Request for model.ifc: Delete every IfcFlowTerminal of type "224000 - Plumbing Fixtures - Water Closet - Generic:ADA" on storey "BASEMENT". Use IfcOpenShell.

First a look at what the model holds.

```python
import ifcopenshell
import ifcopenshell.util.element

model = ifcopenshell.open("model.ifc")
print(model.schema)
storey = next(s for s in model.by_type("IfcBuildingStorey") if s.Name == "BASEMENT")
terminals = [e for e in ifcopenshell.util.element.get_decomposition(storey) if e.is_a("IfcFlowTerminal")]
seen = {}
for e in terminals:
    element_type = ifcopenshell.util.element.get_type(e)
    name = element_type.Name if element_type not in (None, e) else None
    seen[name] = seen.get(name, 0) + 1
for name, count in sorted(seen.items(), key=str):
    print(count, "x", name)
```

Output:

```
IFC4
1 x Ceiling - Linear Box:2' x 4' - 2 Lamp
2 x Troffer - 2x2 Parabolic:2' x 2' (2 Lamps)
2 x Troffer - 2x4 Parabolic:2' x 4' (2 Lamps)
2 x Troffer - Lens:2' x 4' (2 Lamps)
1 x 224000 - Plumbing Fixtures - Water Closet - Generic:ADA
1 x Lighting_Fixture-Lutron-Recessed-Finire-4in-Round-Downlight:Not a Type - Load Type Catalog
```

```python
import ifcopenshell
import ifcopenshell.api.root
import ifcopenshell.util.element

model = ifcopenshell.open("model.ifc")

storey = next(s for s in model.by_type("IfcBuildingStorey") if s.Name == "BASEMENT")
terminals = [e for e in ifcopenshell.util.element.get_decomposition(storey) if e.is_a("IfcFlowTerminal")]
targets = [e for e in terminals if (t := ifcopenshell.util.element.get_type(e)) not in (None, e) and t.Name == "224000 - Plumbing Fixtures - Water Closet - Generic:ADA"]

for e in targets:
    ifcopenshell.api.root.remove_product(model, product=e)
print(len(targets), "removed")

model.write("model_v2.ifc")
```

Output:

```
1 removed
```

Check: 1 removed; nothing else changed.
